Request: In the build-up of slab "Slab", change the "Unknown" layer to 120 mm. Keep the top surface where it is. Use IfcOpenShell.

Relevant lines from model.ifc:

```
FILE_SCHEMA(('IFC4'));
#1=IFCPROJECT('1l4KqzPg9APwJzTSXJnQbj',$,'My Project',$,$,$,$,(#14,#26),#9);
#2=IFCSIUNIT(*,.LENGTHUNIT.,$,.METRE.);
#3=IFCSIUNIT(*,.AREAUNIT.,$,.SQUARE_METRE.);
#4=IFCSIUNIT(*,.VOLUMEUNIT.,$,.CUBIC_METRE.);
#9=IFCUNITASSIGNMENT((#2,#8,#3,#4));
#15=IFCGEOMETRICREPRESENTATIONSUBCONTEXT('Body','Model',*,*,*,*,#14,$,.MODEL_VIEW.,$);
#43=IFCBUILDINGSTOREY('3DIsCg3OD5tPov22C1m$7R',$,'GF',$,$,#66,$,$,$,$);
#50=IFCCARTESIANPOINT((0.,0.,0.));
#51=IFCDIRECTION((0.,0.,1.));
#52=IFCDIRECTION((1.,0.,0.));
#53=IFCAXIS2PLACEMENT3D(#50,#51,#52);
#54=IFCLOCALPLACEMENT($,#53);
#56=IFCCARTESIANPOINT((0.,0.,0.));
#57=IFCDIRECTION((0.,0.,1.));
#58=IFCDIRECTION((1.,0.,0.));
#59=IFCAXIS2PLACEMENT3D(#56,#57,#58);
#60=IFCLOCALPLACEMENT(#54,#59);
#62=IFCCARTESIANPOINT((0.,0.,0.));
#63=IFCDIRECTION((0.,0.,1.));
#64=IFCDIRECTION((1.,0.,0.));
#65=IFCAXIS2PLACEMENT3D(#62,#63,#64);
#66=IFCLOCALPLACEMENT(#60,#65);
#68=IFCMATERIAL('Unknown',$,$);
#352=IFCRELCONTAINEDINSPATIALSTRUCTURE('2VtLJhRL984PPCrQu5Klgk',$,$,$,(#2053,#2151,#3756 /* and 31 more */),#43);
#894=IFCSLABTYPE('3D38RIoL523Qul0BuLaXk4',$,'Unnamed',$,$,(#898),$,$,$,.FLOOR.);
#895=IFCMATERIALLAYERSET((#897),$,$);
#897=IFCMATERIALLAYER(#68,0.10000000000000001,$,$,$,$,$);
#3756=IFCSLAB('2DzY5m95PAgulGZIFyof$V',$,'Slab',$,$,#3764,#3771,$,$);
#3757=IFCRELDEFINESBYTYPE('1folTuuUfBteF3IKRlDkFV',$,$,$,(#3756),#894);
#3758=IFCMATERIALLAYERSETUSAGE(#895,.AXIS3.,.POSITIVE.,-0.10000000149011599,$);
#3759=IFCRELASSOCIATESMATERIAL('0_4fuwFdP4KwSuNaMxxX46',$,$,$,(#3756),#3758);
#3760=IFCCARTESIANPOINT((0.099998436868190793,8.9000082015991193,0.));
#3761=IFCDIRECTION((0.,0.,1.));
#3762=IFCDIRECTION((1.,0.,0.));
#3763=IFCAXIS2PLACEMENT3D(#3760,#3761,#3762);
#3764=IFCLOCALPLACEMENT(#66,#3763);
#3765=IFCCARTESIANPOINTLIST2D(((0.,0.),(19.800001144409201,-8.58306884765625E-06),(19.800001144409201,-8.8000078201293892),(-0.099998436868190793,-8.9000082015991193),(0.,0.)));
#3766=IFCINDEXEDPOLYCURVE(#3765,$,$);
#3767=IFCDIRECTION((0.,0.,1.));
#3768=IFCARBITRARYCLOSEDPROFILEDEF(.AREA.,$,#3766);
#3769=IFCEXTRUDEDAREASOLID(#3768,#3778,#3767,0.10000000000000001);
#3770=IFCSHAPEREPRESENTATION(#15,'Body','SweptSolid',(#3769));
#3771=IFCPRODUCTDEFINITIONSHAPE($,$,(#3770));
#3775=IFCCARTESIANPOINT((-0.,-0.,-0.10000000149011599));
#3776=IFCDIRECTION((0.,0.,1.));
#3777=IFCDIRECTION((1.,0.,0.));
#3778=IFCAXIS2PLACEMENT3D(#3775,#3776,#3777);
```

```python
import ifcopenshell
import ifcopenshell.util.element
import ifcopenshell.util.representation
import ifcopenshell.util.unit

model = ifcopenshell.open("model.ifc")
unit_scale = ifcopenshell.util.unit.calculate_unit_scale(model)

layer_set = model.by_id(895)
layer = next(l for l in layer_set.MaterialLayers if l.Material and l.Material.Name == "Unknown")
change = 0.12 / unit_scale - layer.LayerThickness
layer.LayerThickness += change

# Geometry does not follow the layer set by itself.
slabs = [e for e in ifcopenshell.util.element.get_elements_by_material(model, layer_set) if e.is_a("IfcSlab")]
for slab in sorted(slabs, key=lambda e: e.id()):
    body = ifcopenshell.util.representation.get_representation(slab, "Model", "Body")
    solid = body.Items[0]
    old_depth = solid.Depth
    solid.Depth += change
    # Extruded upwards: lower the start of the extrusion so the top stays.
    x, y, z = solid.Position.Location.Coordinates
    solid.Position.Location = model.createIfcCartesianPoint((x, y, z - change))
    print(slab.id(), f"{old_depth:g} -> {solid.Depth:g}")

# The layers are counted up from the underside, which has moved.
for usage in {ifcopenshell.util.element.get_material(slab) for slab in slabs}:
    usage.OffsetFromReferenceLine -= change

model.write("model_rev.ifc")
```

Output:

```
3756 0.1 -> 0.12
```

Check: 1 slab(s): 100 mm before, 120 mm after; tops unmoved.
